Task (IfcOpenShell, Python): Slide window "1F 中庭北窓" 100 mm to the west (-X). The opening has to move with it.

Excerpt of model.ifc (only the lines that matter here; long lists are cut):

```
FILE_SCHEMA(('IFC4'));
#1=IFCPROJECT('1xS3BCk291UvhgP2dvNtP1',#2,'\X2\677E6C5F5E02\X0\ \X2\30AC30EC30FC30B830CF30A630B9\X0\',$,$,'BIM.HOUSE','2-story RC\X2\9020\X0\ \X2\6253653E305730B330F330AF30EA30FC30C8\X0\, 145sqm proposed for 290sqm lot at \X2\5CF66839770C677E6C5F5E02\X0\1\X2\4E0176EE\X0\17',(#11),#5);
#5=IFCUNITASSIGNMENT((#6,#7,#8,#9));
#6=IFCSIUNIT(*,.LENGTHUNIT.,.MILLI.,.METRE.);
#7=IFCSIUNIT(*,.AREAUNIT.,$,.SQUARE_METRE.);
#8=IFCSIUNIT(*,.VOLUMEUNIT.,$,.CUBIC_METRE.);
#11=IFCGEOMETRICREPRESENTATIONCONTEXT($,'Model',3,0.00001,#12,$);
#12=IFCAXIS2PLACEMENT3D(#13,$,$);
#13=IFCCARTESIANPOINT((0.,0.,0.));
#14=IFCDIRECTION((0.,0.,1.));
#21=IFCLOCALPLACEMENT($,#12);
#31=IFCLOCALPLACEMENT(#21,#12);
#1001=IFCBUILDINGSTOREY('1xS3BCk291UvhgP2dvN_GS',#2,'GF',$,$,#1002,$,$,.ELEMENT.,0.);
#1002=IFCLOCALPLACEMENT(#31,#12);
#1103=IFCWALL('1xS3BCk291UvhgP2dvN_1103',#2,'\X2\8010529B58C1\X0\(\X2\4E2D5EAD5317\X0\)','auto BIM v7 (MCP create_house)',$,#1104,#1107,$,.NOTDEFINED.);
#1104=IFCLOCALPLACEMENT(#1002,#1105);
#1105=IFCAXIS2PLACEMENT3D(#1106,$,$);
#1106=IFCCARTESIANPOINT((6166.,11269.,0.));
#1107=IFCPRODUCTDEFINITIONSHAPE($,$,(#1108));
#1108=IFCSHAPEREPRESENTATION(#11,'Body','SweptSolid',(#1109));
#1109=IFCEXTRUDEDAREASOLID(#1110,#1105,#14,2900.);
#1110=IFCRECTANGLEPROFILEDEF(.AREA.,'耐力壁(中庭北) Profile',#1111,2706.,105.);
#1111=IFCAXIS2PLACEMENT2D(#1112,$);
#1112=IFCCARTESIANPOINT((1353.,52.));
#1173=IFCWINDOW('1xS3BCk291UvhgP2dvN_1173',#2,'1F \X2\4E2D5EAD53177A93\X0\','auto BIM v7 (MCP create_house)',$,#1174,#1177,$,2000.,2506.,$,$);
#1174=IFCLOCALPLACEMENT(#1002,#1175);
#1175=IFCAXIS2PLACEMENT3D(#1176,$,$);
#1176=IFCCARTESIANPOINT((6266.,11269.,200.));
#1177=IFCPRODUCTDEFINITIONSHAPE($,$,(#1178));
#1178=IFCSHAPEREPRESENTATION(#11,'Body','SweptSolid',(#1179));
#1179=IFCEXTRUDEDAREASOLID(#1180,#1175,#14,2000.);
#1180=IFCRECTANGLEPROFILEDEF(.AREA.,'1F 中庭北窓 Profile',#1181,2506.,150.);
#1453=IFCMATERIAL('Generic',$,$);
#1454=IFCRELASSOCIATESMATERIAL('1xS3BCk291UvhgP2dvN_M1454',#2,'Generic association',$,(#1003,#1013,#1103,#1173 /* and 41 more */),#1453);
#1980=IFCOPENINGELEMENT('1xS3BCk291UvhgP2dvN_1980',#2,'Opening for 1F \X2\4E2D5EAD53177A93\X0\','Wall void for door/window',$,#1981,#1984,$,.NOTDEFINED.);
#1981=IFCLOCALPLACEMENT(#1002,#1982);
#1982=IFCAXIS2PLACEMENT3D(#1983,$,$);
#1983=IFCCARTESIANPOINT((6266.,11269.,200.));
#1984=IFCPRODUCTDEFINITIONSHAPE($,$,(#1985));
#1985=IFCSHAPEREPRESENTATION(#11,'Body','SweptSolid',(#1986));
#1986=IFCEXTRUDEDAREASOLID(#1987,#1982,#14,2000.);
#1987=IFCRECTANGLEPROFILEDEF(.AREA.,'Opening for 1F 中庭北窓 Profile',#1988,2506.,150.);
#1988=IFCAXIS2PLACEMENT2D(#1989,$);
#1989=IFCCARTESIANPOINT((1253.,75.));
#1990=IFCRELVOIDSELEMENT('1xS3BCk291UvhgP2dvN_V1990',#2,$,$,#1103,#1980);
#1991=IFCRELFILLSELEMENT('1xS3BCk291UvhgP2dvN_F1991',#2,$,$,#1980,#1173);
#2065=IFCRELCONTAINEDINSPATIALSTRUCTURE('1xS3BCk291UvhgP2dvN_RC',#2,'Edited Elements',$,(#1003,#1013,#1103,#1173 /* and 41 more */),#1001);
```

```python
import ifcopenshell
import ifcopenshell.api.geometry
import ifcopenshell.util.placement
import ifcopenshell.util.unit

model = ifcopenshell.open("model.ifc")
unit_scale = ifcopenshell.util.unit.calculate_unit_scale(model)

window = model.by_id(1173)
opening = window.FillsVoids[0].RelatingOpeningElement
wall = opening.VoidsElements[0].RelatingBuildingElement

wall_matrix = ifcopenshell.util.placement.get_local_placement(wall.ObjectPlacement)
shift = wall_matrix[:3, 0] * -0.1 / unit_scale
before = ifcopenshell.util.placement.get_local_placement(window.ObjectPlacement)[:3, 3].copy()

# The window is not placed relative to its opening, so move both.
for product in (opening, window):
    matrix = ifcopenshell.util.placement.get_local_placement(product.ObjectPlacement)
    matrix[:3, 3] += shift
    ifcopenshell.api.geometry.edit_object_placement(model, product=product, matrix=matrix, is_si=False)

after = ifcopenshell.util.placement.get_local_placement(window.ObjectPlacement)[:3, 3]
print("window moved by", (after - before).round(3) + 0.0)

model.write("model_edited.ifc")
```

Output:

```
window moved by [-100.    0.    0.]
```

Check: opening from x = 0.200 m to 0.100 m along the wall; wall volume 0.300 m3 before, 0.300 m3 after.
